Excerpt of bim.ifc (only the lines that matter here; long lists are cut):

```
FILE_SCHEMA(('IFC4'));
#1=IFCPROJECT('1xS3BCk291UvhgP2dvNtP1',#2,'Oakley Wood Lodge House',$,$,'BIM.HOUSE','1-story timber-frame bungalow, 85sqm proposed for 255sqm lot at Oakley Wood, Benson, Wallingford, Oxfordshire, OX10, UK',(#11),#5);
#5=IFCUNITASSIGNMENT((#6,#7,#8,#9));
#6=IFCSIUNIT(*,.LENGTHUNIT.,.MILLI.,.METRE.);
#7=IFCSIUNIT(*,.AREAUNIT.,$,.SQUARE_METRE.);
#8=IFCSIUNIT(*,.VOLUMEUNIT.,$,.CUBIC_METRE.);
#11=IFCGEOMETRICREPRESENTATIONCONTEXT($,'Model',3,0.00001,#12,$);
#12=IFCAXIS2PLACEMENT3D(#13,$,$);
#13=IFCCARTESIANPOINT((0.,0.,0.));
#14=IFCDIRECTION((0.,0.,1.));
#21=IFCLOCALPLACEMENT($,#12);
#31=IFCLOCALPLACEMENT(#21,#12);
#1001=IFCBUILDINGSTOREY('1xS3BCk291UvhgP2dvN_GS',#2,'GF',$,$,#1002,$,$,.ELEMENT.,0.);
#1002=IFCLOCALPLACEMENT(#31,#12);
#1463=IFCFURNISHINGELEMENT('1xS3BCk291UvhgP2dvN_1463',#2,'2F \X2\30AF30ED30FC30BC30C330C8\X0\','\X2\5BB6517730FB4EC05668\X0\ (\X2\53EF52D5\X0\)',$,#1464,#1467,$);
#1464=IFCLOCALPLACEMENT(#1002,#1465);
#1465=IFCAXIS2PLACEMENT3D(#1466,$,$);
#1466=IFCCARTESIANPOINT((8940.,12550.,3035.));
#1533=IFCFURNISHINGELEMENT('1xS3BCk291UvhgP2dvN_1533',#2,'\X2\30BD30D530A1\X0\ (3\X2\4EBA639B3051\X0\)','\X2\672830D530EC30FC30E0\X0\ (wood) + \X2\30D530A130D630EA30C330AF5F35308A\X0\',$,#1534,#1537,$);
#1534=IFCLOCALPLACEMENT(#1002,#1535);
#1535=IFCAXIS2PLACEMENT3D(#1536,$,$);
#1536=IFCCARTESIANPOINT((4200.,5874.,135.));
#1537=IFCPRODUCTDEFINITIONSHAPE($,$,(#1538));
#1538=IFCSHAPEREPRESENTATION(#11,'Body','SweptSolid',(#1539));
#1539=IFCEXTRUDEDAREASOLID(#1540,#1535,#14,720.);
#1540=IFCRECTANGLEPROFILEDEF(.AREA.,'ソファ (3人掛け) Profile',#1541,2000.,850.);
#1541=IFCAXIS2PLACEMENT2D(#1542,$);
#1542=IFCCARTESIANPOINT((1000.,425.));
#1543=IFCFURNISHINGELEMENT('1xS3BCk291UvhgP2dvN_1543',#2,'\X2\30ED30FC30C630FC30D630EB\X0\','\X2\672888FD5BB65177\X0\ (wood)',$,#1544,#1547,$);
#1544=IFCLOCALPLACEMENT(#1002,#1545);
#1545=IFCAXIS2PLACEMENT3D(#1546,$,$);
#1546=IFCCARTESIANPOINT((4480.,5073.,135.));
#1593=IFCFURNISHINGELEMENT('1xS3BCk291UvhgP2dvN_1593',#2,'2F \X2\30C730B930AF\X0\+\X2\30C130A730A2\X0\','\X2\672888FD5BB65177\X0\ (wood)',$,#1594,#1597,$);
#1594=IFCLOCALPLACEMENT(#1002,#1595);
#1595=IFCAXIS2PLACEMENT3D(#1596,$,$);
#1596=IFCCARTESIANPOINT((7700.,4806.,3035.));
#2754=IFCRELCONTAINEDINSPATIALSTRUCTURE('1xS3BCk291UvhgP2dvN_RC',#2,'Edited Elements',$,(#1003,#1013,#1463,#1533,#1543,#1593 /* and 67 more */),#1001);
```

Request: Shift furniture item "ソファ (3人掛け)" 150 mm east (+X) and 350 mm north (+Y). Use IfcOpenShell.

```python
import ifcopenshell
import ifcopenshell.api.geometry
import ifcopenshell.util.placement
import ifcopenshell.util.unit

model = ifcopenshell.open("bim.ifc")
unit_scale = ifcopenshell.util.unit.calculate_unit_scale(model)

item = model.by_id(1533)
matrix = ifcopenshell.util.placement.get_local_placement(item.ObjectPlacement)
matrix[0, 3] += 0.15 / unit_scale
matrix[1, 3] += 0.35 / unit_scale
ifcopenshell.api.geometry.edit_object_placement(model, product=item, matrix=matrix, is_si=False)

print(ifcopenshell.util.placement.get_local_placement(item.ObjectPlacement).round(3) + 0.0)

model.write("bim_edited.ifc")
```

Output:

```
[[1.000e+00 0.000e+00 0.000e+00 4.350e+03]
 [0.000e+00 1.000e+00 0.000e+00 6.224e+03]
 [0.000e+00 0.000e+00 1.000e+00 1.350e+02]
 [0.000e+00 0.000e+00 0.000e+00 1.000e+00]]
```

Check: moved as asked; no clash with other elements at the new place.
